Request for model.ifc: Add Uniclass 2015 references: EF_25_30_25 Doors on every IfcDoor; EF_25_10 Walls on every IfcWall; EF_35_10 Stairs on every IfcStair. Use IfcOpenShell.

First a look at what the model holds.

```python
import ifcopenshell

model = ifcopenshell.open("model.ifc")
print(model.schema)
print("classifications:", [c.Name for c in model.by_type("IfcClassification")])
for ifc_class in ("IfcDoor", "IfcRoof", "IfcStair", "IfcWall", "IfcWindow"):
    print(ifc_class, len(model.by_type(ifc_class)))
```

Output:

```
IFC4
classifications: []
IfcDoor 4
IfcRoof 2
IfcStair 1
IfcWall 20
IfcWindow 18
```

```python
import ifcopenshell
import ifcopenshell.api.classification

model = ifcopenshell.open("model.ifc")

system = ifcopenshell.api.classification.add_classification(model, classification="Uniclass 2015")

codes = {
    "IfcDoor": ("EF_25_30_25", "Doors"),
    "IfcWall": ("EF_25_10", "Walls"),
    "IfcStair": ("EF_35_10", "Stairs"),
}
for ifc_class, (code, name) in codes.items():
    products = model.by_type(ifc_class)
    ifcopenshell.api.classification.add_reference(
        model, products=products, classification=system, identification=code, name=name
    )
    print(code, len(products))

model.write("model_updated.ifc")
```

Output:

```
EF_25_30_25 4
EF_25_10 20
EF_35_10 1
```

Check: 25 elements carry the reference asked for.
